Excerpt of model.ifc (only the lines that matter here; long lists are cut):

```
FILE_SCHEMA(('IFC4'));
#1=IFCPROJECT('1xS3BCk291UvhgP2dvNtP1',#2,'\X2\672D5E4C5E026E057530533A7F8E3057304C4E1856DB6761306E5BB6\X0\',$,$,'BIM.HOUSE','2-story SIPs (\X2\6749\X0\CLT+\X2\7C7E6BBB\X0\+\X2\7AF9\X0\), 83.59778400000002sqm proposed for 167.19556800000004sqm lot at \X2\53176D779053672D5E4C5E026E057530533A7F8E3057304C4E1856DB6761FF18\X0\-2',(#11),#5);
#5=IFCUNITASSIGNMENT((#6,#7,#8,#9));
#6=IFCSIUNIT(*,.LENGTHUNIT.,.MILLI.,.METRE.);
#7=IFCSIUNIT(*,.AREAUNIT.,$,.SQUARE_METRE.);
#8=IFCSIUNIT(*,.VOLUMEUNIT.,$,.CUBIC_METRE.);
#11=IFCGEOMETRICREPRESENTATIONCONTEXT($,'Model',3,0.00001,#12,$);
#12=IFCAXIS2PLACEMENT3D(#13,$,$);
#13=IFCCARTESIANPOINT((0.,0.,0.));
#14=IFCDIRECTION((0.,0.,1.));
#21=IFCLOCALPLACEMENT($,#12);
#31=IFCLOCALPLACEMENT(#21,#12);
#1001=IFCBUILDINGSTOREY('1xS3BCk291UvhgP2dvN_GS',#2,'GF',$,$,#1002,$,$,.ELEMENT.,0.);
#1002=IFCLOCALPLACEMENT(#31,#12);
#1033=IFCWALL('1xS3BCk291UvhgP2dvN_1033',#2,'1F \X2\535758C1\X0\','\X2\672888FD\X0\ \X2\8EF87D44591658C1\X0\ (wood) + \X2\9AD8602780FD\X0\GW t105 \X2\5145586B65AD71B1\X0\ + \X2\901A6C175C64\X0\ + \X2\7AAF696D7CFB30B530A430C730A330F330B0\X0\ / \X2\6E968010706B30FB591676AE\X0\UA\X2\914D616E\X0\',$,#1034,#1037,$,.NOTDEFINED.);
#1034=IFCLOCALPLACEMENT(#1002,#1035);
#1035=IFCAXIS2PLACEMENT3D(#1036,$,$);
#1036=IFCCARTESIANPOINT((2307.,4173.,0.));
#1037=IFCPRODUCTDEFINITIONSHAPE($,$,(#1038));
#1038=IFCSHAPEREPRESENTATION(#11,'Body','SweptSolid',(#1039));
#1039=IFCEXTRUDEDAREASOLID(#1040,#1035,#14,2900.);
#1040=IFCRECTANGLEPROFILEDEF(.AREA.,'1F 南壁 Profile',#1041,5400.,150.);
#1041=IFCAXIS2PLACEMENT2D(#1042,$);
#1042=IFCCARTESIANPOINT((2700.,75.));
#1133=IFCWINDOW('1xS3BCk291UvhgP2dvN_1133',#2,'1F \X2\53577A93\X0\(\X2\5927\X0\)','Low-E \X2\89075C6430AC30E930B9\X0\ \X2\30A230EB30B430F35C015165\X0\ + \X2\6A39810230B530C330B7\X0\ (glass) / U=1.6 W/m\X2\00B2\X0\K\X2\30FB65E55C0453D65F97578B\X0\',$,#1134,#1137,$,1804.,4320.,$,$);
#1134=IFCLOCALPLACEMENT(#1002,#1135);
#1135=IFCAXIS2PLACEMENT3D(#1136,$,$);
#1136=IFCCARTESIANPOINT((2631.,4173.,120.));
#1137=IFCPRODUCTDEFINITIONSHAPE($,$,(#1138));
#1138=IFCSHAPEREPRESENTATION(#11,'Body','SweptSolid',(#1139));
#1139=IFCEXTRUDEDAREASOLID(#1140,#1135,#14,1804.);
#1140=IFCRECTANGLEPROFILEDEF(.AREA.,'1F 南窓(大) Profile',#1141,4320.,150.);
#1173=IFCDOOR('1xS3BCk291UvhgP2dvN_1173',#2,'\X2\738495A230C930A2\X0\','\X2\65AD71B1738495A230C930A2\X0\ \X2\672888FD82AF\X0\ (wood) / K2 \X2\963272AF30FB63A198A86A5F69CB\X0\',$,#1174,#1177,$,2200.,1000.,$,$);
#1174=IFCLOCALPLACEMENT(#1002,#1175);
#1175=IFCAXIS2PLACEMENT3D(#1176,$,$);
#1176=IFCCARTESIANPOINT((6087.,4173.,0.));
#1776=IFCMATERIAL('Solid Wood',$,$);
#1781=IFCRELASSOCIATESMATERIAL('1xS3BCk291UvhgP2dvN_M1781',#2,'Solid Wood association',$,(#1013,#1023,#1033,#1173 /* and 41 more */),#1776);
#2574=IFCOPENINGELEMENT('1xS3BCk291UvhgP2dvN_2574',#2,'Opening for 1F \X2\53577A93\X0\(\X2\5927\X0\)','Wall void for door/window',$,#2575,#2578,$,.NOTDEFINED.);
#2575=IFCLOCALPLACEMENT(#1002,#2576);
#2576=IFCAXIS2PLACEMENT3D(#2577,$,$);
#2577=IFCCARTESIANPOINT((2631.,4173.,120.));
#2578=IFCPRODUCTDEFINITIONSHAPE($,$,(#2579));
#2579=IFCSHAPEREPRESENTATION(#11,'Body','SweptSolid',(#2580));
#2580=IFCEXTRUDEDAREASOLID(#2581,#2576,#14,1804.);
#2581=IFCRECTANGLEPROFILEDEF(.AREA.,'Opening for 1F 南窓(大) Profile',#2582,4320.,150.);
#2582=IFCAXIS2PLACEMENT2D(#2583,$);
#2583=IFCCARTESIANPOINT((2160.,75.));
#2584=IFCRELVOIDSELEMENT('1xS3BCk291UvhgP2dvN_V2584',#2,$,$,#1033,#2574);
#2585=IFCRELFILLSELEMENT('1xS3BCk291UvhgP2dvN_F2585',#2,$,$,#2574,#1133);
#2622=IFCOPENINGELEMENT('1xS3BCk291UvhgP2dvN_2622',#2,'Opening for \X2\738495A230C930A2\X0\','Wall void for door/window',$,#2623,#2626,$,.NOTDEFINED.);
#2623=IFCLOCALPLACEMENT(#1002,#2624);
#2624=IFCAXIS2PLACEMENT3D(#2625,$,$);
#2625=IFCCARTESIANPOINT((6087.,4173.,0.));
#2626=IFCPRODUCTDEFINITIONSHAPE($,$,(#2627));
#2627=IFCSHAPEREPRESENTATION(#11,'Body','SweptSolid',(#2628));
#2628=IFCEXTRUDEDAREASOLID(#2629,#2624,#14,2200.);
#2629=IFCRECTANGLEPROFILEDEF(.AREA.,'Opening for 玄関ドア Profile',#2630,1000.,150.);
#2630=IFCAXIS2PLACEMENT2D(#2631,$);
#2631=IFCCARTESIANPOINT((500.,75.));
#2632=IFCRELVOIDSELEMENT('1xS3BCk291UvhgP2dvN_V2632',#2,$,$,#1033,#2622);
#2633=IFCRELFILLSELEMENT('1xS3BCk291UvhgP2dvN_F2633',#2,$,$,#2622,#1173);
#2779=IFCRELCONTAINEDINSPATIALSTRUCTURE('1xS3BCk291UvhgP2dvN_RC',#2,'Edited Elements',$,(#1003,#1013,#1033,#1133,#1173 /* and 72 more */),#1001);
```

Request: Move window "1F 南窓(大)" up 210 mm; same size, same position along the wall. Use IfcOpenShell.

```python
import numpy as np
import ifcopenshell
import ifcopenshell.api.geometry
import ifcopenshell.util.placement
import ifcopenshell.util.unit

model = ifcopenshell.open("model.ifc")
unit_scale = ifcopenshell.util.unit.calculate_unit_scale(model)

window = model.by_id(1133)
opening = window.FillsVoids[0].RelatingOpeningElement
dz = 0.21 / unit_scale

shift = np.array([0.0, 0.0, dz])
# The window is not placed relative to its opening, so move both.
for product in (opening, window):
    matrix = ifcopenshell.util.placement.get_local_placement(product.ObjectPlacement)
    matrix[:3, 3] += shift
    ifcopenshell.api.geometry.edit_object_placement(model, product=product, matrix=matrix, is_si=False)

print(f"moved by {dz * unit_scale:+.3f} m")

model.write("model-out.ifc")
```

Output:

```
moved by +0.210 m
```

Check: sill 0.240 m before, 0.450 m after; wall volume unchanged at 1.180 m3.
